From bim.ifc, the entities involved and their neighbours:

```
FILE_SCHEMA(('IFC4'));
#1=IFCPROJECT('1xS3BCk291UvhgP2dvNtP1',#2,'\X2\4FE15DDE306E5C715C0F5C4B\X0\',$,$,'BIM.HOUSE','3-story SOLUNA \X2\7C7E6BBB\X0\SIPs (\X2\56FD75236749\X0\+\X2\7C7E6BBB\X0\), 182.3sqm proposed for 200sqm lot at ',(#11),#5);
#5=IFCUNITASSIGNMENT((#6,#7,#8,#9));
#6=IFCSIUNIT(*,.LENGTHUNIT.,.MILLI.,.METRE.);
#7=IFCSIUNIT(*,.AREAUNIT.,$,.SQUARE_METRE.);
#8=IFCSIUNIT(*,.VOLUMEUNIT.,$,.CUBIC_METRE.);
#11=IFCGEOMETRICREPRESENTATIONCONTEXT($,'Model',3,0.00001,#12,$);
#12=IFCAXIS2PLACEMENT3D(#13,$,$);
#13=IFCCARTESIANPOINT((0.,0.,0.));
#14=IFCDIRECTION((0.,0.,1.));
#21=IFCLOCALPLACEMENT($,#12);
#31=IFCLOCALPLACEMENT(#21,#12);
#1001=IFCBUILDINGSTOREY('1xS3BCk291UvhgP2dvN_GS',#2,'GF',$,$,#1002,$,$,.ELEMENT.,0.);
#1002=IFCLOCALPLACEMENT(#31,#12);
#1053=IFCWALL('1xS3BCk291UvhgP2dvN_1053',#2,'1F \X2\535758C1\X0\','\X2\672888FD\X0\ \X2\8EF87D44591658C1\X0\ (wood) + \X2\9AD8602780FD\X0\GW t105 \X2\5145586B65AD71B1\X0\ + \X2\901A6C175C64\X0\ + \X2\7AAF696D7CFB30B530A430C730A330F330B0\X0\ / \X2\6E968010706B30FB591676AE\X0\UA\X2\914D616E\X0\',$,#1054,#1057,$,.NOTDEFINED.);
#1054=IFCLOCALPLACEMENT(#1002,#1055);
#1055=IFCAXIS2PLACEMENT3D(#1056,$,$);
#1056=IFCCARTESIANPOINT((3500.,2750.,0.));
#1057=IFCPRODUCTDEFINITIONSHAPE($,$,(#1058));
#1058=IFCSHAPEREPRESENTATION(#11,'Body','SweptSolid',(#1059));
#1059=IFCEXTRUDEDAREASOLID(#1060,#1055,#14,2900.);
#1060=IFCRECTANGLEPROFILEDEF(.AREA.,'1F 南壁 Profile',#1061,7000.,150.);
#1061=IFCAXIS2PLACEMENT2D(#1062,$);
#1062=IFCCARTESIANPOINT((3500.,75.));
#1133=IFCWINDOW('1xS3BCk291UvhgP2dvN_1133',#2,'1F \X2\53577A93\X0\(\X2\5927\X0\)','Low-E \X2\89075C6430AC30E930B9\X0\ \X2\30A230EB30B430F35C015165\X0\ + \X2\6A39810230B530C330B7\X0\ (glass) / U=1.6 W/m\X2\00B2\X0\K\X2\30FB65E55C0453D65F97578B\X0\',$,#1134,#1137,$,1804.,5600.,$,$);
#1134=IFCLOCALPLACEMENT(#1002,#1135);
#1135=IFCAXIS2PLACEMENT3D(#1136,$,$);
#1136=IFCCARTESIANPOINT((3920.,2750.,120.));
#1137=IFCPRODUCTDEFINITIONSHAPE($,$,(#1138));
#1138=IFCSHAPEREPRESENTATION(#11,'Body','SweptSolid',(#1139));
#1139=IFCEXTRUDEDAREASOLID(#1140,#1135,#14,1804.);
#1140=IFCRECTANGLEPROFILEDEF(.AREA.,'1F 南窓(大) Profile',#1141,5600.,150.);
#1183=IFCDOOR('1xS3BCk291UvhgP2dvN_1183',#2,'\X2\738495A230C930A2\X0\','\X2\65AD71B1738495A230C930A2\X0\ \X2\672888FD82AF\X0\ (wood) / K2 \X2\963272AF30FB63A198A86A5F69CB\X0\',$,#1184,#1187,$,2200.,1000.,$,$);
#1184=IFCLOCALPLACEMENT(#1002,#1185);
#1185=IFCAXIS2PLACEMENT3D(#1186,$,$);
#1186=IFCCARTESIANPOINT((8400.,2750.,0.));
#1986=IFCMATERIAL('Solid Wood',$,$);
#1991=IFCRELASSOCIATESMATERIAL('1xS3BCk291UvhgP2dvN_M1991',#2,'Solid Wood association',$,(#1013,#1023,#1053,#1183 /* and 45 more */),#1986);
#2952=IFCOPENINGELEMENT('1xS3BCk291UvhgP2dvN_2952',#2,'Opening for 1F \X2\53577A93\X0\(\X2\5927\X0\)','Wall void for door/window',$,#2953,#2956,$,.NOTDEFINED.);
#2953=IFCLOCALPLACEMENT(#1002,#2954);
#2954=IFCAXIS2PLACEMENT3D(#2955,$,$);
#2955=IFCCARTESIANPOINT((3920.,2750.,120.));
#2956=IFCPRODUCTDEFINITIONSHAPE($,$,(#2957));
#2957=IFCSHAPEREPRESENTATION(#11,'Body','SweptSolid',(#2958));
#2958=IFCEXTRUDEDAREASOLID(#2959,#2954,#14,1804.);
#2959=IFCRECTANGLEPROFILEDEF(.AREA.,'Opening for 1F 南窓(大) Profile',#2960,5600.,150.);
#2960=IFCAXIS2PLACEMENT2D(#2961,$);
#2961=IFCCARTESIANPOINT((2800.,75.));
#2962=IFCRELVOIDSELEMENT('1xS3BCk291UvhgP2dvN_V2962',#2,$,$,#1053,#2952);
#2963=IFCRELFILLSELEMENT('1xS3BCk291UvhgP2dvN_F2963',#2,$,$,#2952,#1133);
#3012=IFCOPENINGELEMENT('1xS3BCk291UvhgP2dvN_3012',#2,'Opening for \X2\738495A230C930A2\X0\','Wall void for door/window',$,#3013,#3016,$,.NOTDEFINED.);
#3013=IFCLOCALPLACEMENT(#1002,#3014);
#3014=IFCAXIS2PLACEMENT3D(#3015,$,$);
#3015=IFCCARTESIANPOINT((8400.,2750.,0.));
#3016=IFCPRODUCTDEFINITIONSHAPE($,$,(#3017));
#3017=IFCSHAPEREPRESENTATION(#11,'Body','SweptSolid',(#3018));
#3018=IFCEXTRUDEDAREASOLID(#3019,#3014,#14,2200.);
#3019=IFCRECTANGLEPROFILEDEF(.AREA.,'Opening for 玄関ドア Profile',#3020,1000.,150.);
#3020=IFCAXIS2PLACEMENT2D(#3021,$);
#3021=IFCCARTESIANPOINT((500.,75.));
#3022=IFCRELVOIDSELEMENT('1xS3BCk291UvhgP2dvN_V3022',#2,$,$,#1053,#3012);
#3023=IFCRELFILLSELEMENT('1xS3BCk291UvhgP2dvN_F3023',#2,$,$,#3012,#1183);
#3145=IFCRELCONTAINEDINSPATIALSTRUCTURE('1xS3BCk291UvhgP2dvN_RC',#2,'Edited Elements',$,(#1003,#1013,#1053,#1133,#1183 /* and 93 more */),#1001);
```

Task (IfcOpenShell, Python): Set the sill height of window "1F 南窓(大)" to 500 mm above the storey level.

```python
import numpy as np
import ifcopenshell
import ifcopenshell.api.geometry
import ifcopenshell.geom
import ifcopenshell.util.element
import ifcopenshell.util.placement
import ifcopenshell.util.shape
import ifcopenshell.util.unit

model = ifcopenshell.open("bim.ifc")
unit_scale = ifcopenshell.util.unit.calculate_unit_scale(model)

window = model.by_id(1133)
opening = window.FillsVoids[0].RelatingOpeningElement
storey = ifcopenshell.util.element.get_container(window, ifc_class="IfcBuildingStorey")
level = ifcopenshell.util.placement.get_local_placement(storey.ObjectPlacement)[2, 3]

# The opening's origin need not be at the sill, so measure its lowest point.
shape = ifcopenshell.geom.create_shape(ifcopenshell.geom.settings(), opening)
bottom = ifcopenshell.util.shape.get_shape_bottom_elevation(shape, shape.geometry) / unit_scale
dz = level + 0.5 / unit_scale - bottom

shift = np.array([0.0, 0.0, dz])
# The window is not placed relative to its opening, so move both.
for product in (opening, window):
    matrix = ifcopenshell.util.placement.get_local_placement(product.ObjectPlacement)
    matrix[:3, 3] += shift
    ifcopenshell.api.geometry.edit_object_placement(model, product=product, matrix=matrix, is_si=False)

print(f"moved by {dz * unit_scale:+.3f} m")

model.write("bim_rev.ifc")
```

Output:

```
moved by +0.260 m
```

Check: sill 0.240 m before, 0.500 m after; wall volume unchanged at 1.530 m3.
